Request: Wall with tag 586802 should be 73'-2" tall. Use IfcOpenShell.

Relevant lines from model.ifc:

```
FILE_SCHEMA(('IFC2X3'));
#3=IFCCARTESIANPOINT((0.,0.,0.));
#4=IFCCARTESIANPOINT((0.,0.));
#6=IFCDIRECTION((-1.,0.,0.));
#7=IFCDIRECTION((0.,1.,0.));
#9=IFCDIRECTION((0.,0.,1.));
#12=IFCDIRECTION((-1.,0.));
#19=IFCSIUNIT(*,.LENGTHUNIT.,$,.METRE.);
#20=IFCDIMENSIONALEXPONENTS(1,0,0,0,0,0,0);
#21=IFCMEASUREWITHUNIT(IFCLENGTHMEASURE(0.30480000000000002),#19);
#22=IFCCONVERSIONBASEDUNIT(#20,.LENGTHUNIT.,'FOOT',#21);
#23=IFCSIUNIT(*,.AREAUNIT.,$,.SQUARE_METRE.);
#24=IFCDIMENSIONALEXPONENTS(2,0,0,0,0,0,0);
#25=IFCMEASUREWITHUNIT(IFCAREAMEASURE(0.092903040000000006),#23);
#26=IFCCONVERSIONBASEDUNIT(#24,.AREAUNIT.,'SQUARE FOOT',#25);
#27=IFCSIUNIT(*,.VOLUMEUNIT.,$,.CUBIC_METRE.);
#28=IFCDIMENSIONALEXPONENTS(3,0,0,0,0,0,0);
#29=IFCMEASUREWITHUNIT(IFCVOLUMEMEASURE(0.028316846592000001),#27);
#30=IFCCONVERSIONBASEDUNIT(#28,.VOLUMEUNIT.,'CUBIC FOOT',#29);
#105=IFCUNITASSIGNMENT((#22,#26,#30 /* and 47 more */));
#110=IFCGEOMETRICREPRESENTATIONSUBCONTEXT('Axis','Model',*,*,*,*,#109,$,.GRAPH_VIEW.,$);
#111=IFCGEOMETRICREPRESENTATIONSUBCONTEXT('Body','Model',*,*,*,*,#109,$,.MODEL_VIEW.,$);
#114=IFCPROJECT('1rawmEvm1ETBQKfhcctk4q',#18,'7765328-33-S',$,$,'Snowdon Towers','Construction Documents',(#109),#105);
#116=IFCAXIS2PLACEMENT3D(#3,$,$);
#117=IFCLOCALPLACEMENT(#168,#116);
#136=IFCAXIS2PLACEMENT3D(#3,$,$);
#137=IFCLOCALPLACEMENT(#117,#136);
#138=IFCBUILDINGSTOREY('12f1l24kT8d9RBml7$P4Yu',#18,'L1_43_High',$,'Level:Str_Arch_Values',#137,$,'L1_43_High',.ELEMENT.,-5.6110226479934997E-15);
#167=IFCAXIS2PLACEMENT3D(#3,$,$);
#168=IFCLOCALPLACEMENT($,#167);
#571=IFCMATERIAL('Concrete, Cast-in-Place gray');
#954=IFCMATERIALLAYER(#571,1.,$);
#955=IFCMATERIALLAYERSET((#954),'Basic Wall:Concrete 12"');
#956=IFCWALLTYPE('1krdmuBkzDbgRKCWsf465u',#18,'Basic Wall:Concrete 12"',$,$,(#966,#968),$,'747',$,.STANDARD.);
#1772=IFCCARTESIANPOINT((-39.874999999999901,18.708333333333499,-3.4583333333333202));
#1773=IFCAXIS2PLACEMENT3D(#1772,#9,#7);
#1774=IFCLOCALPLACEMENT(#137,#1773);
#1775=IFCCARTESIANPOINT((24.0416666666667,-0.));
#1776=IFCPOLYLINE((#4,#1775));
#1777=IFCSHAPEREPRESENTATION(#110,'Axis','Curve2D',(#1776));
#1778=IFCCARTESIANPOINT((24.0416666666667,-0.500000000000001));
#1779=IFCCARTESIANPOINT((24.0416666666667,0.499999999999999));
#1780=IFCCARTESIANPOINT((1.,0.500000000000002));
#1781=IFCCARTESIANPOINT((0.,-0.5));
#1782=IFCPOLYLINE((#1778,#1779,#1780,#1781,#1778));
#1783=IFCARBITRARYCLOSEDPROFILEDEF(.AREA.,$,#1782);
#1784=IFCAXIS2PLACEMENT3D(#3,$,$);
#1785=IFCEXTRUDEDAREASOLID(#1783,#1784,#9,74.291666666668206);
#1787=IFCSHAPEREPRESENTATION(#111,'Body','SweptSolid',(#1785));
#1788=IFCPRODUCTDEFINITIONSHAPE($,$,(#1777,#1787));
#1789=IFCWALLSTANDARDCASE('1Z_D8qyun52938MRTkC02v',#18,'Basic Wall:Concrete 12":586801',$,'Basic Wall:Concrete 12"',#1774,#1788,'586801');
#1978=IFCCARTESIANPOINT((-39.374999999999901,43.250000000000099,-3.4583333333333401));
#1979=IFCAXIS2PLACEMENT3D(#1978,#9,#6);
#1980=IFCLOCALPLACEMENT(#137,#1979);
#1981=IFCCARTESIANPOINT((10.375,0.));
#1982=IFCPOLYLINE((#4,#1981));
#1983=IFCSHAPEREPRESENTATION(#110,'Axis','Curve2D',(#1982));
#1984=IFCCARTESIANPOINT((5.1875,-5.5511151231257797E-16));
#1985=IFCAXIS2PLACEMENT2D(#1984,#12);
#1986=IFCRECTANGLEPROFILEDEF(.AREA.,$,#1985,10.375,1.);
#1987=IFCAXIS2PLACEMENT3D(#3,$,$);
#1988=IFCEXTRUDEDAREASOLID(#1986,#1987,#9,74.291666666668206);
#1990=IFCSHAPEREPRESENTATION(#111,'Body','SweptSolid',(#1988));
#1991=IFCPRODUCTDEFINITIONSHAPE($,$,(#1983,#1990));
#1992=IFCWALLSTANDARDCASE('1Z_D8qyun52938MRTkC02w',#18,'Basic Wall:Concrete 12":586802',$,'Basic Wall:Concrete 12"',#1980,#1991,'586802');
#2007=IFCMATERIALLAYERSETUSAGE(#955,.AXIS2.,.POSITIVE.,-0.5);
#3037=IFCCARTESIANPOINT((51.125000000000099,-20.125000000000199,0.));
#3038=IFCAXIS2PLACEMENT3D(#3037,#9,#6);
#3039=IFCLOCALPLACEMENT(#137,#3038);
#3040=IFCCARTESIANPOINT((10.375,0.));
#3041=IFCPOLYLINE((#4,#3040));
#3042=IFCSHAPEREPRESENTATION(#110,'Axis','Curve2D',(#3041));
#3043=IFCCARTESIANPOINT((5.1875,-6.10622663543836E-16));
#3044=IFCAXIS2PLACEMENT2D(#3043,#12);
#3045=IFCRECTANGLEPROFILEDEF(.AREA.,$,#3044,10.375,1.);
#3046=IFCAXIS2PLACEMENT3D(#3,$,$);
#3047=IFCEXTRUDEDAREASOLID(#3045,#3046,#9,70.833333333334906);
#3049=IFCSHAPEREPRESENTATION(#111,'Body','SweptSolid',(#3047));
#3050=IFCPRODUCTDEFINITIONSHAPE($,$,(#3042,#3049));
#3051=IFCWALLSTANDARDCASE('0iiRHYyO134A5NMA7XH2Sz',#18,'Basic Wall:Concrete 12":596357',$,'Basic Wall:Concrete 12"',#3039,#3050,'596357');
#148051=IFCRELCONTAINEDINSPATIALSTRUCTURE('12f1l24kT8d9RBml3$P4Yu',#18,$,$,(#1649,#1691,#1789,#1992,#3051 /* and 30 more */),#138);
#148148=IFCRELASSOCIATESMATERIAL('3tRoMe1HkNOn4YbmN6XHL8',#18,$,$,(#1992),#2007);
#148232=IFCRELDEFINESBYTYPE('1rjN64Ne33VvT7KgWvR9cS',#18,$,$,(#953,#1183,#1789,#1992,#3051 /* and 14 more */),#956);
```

```python
import ifcopenshell
import ifcopenshell.geom
import ifcopenshell.util.representation
import ifcopenshell.util.shape
import ifcopenshell.util.unit

model = ifcopenshell.open("model.ifc")
unit_scale = ifcopenshell.util.unit.calculate_unit_scale(model)
settings = ifcopenshell.geom.settings()


def volume(element):
    """Net volume in cubic metres, openings subtracted."""
    shape = ifcopenshell.geom.create_shape(settings, element)
    return ifcopenshell.util.shape.get_volume(shape.geometry)


wall = model.by_guid("1Z_D8qyun52938MRTkC02w")
before = volume(wall)

body = ifcopenshell.util.representation.get_representation(wall, "Model", "Body")
solid = body.Items[0]
old_height = solid.Depth
solid.Depth = 878 * 0.0254 / unit_scale
after = volume(wall)

print(f"height {old_height:g} -> {solid.Depth:g}, volume {before:.3f} -> {after:.3f} m3")

model.write("model_rev.ifc")
```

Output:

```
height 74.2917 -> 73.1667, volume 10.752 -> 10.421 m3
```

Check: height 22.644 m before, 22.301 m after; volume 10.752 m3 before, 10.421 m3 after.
